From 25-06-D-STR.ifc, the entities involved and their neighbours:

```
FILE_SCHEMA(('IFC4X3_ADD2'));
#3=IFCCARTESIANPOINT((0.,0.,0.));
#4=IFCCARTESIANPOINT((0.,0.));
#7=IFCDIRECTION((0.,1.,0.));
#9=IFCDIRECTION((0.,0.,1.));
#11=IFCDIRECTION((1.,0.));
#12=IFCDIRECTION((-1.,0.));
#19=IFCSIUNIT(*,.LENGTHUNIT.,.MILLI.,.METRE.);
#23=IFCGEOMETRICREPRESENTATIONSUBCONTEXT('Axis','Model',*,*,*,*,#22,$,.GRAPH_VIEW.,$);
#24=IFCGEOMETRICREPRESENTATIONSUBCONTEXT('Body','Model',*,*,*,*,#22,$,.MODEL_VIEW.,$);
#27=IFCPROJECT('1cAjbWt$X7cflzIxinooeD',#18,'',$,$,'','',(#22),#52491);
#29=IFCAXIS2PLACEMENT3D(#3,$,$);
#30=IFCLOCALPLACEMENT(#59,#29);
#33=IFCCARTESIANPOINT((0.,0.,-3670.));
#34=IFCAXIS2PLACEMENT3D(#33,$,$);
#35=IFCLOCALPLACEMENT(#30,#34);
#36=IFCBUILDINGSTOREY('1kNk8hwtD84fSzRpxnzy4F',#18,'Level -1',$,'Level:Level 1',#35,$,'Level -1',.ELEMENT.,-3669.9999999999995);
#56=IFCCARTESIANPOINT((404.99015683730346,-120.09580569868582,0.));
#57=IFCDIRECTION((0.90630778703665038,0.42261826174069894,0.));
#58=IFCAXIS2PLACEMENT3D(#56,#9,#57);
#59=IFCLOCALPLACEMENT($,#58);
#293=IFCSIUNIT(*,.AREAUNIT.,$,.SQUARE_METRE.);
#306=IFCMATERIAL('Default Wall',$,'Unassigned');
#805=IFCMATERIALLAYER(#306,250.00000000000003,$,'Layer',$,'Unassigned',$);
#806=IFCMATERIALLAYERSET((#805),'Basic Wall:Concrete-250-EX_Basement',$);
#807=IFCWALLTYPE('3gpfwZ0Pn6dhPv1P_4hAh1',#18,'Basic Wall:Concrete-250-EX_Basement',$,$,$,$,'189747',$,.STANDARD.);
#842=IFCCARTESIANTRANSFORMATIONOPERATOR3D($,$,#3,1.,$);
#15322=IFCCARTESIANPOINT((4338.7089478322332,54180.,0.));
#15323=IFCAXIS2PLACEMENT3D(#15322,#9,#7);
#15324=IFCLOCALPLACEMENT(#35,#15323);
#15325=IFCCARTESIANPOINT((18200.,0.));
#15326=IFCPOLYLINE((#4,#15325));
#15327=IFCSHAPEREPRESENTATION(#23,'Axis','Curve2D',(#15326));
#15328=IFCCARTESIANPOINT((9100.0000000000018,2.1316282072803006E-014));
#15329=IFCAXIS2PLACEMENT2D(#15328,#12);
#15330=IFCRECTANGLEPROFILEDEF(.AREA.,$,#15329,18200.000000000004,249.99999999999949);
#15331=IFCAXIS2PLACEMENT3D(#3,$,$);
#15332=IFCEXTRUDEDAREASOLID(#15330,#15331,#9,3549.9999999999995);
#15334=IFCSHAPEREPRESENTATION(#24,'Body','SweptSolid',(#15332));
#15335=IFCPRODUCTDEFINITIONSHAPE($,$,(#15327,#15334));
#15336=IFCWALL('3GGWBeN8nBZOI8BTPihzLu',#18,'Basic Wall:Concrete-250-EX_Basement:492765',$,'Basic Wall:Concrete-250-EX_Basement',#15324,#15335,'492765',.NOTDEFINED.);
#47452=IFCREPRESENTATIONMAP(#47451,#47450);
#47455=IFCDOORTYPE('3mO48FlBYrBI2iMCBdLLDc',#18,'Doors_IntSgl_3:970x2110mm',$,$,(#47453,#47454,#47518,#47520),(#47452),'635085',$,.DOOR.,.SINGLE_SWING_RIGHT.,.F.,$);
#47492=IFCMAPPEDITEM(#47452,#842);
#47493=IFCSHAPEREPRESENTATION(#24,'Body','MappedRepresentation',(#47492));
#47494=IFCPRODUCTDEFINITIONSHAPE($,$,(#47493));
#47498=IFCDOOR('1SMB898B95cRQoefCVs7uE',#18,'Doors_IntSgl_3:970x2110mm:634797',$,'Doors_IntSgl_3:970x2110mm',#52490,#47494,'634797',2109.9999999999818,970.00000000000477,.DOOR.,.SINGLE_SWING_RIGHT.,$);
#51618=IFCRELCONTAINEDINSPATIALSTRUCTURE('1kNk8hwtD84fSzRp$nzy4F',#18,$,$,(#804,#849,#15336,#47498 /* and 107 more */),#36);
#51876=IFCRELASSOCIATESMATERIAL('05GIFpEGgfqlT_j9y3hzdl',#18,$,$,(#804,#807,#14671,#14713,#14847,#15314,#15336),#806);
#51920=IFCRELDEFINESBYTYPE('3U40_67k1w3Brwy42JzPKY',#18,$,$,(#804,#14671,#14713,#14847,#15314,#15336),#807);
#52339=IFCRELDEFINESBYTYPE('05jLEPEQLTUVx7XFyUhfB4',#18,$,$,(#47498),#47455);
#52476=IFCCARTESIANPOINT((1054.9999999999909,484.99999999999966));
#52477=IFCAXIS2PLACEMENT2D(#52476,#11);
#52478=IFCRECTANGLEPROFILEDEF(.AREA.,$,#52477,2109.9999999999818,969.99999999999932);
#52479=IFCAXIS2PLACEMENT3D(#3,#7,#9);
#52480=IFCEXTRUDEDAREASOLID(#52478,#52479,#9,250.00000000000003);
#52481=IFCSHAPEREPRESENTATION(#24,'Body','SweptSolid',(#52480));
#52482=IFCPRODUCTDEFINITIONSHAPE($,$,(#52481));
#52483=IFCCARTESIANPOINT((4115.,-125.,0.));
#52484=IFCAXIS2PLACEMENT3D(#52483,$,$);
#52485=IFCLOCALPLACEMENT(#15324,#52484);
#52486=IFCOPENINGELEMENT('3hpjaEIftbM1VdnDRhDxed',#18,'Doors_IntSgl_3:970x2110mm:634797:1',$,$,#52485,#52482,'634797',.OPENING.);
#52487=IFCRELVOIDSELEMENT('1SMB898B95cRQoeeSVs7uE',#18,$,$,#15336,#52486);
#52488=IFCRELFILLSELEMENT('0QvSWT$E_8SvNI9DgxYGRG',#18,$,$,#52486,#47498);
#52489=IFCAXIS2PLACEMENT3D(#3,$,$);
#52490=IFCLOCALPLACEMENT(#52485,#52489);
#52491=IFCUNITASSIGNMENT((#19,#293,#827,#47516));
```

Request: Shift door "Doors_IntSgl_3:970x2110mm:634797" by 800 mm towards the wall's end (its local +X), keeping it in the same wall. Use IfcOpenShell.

```python
import ifcopenshell
import ifcopenshell.api.geometry
import ifcopenshell.util.placement

model = ifcopenshell.open("25-06-D-STR.ifc")

door = model.by_guid("1SMB898B95cRQoefCVs7uE")
opening = door.FillsVoids[0].RelatingOpeningElement
wall = opening.VoidsElements[0].RelatingBuildingElement

wall_matrix = ifcopenshell.util.placement.get_local_placement(wall.ObjectPlacement)
shift = wall_matrix[:3, 0] * 800.0
before = ifcopenshell.util.placement.get_local_placement(door.ObjectPlacement)[:3, 3].copy()

# The door is placed relative to its opening, so it follows when the opening moves.
matrix = ifcopenshell.util.placement.get_local_placement(opening.ObjectPlacement)
matrix[:3, 3] += shift
ifcopenshell.api.geometry.edit_object_placement(
    model, product=opening, matrix=matrix, is_si=False, should_transform_children=True
)

after = ifcopenshell.util.placement.get_local_placement(door.ObjectPlacement)[:3, 3]
print("door moved by", (after - before).round(3) + 0.0)

model.write("25-06-D-STR_updated.ifc")
```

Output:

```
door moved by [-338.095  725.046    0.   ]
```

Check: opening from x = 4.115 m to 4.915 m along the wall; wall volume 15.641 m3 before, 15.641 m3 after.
